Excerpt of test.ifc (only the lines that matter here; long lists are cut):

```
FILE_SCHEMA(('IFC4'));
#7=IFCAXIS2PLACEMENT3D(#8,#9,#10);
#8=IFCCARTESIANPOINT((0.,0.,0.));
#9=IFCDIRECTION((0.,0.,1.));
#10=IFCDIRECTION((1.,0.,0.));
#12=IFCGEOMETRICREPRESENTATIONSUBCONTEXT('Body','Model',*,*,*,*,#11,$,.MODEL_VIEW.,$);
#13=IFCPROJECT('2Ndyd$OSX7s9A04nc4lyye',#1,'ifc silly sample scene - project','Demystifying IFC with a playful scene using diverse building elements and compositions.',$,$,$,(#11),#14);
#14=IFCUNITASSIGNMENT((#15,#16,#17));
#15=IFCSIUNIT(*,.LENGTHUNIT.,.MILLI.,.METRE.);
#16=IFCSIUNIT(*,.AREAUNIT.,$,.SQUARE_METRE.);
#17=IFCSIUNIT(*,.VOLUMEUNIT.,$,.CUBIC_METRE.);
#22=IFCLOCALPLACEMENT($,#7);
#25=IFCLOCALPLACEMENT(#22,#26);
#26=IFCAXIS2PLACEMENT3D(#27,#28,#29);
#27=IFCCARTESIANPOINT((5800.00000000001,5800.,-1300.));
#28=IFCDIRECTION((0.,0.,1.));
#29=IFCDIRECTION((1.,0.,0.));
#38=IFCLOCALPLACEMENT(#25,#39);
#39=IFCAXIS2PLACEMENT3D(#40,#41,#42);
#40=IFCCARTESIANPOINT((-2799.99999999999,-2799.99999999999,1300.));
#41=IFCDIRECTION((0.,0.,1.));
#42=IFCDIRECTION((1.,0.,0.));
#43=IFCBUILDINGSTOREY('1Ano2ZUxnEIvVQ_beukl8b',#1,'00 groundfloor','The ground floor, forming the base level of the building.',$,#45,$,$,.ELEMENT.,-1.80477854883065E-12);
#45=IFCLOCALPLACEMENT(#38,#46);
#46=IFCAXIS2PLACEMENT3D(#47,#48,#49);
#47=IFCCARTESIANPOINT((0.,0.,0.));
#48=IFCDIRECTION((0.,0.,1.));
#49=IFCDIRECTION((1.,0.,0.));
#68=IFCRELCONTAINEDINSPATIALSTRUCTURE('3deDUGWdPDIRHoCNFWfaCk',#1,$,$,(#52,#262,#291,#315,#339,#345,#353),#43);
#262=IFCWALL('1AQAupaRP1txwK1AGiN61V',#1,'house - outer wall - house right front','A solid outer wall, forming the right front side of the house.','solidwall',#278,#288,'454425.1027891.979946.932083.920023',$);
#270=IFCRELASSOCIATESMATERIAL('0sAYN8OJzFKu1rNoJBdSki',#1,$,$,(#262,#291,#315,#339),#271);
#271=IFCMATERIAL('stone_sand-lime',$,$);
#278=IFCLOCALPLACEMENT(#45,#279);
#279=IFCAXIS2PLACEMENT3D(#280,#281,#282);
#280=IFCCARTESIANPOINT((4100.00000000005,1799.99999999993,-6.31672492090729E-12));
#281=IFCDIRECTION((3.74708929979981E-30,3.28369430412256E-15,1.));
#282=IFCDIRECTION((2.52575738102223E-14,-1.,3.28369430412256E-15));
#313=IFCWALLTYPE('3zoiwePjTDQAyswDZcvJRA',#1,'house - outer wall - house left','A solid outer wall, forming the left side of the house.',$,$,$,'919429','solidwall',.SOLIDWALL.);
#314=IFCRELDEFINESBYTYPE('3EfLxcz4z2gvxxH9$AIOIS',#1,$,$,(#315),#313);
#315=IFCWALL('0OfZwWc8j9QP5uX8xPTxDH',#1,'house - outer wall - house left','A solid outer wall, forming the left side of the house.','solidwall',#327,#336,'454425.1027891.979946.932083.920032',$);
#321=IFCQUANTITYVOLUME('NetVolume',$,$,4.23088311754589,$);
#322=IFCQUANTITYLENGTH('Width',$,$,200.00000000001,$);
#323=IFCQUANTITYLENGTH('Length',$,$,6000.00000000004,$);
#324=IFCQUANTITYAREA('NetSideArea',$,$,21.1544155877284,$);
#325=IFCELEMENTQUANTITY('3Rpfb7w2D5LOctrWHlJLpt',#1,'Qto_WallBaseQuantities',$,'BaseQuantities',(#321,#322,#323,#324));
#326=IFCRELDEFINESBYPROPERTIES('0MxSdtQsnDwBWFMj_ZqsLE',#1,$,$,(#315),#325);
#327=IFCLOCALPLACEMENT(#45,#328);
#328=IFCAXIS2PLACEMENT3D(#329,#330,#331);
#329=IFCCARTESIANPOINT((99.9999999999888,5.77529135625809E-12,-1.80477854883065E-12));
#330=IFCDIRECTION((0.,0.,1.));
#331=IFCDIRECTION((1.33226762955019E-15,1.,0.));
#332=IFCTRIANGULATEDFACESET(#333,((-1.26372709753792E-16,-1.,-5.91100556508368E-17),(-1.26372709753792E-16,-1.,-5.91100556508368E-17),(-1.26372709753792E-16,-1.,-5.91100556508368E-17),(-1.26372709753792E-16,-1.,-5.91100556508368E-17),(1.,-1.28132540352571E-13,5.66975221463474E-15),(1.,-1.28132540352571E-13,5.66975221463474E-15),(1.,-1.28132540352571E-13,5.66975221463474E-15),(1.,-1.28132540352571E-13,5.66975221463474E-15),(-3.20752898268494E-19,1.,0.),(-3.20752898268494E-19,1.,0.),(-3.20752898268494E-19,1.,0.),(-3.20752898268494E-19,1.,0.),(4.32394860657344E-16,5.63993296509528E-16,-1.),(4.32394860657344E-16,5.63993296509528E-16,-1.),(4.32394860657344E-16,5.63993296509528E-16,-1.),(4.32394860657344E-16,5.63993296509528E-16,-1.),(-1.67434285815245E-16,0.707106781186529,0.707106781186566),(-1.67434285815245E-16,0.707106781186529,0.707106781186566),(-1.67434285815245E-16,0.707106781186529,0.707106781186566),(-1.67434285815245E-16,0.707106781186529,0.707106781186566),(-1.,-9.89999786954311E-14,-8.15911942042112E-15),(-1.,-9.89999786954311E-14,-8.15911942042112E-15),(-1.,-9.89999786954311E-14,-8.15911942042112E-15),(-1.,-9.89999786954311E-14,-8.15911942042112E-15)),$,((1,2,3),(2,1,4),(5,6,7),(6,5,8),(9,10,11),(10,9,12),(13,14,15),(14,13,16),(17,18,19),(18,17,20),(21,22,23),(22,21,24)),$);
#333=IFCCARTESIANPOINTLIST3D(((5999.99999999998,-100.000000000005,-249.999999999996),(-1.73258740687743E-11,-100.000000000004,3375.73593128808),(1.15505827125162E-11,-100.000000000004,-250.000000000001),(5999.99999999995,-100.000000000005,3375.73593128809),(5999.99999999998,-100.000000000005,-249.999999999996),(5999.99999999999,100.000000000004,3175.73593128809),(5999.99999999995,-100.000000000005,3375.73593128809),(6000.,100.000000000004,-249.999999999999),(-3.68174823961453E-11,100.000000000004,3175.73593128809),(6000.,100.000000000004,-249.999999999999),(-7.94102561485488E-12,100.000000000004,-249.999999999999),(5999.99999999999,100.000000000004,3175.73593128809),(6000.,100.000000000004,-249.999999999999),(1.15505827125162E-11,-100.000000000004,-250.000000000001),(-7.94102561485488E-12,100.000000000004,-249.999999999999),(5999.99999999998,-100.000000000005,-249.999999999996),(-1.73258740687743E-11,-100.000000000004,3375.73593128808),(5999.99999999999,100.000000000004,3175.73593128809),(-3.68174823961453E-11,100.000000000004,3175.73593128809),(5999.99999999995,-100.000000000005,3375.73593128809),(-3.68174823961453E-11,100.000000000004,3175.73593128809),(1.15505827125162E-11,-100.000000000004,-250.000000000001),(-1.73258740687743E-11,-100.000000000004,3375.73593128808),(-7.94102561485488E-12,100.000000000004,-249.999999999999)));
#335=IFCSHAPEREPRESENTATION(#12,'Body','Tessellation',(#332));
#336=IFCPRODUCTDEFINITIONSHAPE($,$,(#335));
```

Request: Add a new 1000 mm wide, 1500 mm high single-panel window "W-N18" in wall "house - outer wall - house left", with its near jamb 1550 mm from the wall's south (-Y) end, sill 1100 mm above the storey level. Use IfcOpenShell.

```python
import numpy as np
import ifcopenshell
import ifcopenshell.api.feature
import ifcopenshell.api.geometry
import ifcopenshell.api.pset
import ifcopenshell.api.root
import ifcopenshell.api.spatial
import ifcopenshell.geom
import ifcopenshell.util.element
import ifcopenshell.util.placement
import ifcopenshell.util.representation
import ifcopenshell.util.shape
import ifcopenshell.util.unit

model = ifcopenshell.open("test.ifc")
unit_scale = ifcopenshell.util.unit.calculate_unit_scale(model)
area_scale = ifcopenshell.util.unit.calculate_unit_scale(model, "AREAUNIT")
volume_scale = ifcopenshell.util.unit.calculate_unit_scale(model, "VOLUMEUNIT")
settings = ifcopenshell.geom.settings()


def volume(element):
    """Net volume in cubic metres, openings subtracted."""
    shape = ifcopenshell.geom.create_shape(settings, element)
    return ifcopenshell.util.shape.get_volume(shape.geometry)


wall = model.by_guid("0OfZwWc8j9QP5uX8xPTxDH")
storey = ifcopenshell.util.element.get_container(wall, ifc_class="IfcBuildingStorey")
context = ifcopenshell.util.representation.get_context(model, "Model", "Body", "MODEL_VIEW")
before = volume(wall)

width, height, from_end, sill = 1, 1.5, 1.55, 1.1  # metres

# The wall runs along its own X axis, and the end named is its -X end.
wall_shape = ifcopenshell.geom.create_shape(settings, wall)
x, y, z = ifcopenshell.util.shape.get_vertices(wall_shape.geometry).T
start = x.min() + from_end
face, thickness = float(y.min()), float(y.max() - y.min())
wall_matrix = ifcopenshell.util.placement.get_local_placement(wall.ObjectPlacement)
level = ifcopenshell.util.placement.get_local_placement(storey.ObjectPlacement)[2, 3]


def in_wall(x, y):
    """Placement at x, y metres in the wall's axes, at sill height."""
    matrix = wall_matrix.copy()
    matrix[:, 3] = wall_matrix @ np.array([x / unit_scale, y / unit_scale, 0.0, 1.0])
    matrix[2, 3] = level + sill / unit_scale
    return matrix


# Opening: a box that overshoots both wall faces by 50 mm.
opening = ifcopenshell.api.root.create_entity(model, ifc_class="IfcOpeningElement", predefined_type="OPENING")
box = ifcopenshell.api.geometry.add_wall_representation(
    model, context=context, length=width, height=height, thickness=thickness + 0.1
)
ifcopenshell.api.geometry.assign_representation(model, product=opening, representation=box)
ifcopenshell.api.geometry.edit_object_placement(model, product=opening, matrix=in_wall(start, face - 0.05), is_si=False)
ifcopenshell.api.feature.add_feature(model, feature=opening, element=wall)

window = ifcopenshell.api.root.create_entity(model, ifc_class="IfcWindow", name="W-N18", predefined_type="WINDOW")
window.OverallWidth, window.OverallHeight = width / unit_scale, height / unit_scale
window.PartitioningType = "SINGLE_PANEL"
body = ifcopenshell.api.geometry.add_window_representation(
    model,
    context=context,
    overall_width=window.OverallWidth,
    overall_height=window.OverallHeight,
    partition_type="SINGLE_PANEL",
)
ifcopenshell.api.geometry.assign_representation(model, product=window, representation=body)
ifcopenshell.api.spatial.assign_container(model, products=[window], relating_structure=storey)
ifcopenshell.api.feature.add_filling(model, opening=opening, element=window)

# Centre the window in the wall's thickness.
ifcopenshell.api.geometry.edit_object_placement(model, product=window, matrix=in_wall(start, face), is_si=False)
window_shape = ifcopenshell.geom.create_shape(settings, window)
depth = ifcopenshell.util.shape.get_vertices(window_shape.geometry)[:, 1]
offset = face + thickness / 2 - (depth.min() + depth.max()) / 2
ifcopenshell.api.geometry.edit_object_placement(model, product=window, matrix=in_wall(start, offset), is_si=False)

after = volume(wall)

# Update the wall's stored quantities.
qto = model.by_id(ifcopenshell.util.element.get_pset(wall, "Qto_WallBaseQuantities", should_inherit=False)["id"])
ifcopenshell.api.pset.edit_qto(model, qto=qto, properties={
    "NetVolume": after / volume_scale,
    "NetSideArea": after / thickness / area_scale,
})

print(f"wall volume {before:.3f} -> {after:.3f} m3")

model.write("test-out.ifc")
```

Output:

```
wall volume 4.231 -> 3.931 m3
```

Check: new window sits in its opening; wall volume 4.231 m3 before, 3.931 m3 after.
